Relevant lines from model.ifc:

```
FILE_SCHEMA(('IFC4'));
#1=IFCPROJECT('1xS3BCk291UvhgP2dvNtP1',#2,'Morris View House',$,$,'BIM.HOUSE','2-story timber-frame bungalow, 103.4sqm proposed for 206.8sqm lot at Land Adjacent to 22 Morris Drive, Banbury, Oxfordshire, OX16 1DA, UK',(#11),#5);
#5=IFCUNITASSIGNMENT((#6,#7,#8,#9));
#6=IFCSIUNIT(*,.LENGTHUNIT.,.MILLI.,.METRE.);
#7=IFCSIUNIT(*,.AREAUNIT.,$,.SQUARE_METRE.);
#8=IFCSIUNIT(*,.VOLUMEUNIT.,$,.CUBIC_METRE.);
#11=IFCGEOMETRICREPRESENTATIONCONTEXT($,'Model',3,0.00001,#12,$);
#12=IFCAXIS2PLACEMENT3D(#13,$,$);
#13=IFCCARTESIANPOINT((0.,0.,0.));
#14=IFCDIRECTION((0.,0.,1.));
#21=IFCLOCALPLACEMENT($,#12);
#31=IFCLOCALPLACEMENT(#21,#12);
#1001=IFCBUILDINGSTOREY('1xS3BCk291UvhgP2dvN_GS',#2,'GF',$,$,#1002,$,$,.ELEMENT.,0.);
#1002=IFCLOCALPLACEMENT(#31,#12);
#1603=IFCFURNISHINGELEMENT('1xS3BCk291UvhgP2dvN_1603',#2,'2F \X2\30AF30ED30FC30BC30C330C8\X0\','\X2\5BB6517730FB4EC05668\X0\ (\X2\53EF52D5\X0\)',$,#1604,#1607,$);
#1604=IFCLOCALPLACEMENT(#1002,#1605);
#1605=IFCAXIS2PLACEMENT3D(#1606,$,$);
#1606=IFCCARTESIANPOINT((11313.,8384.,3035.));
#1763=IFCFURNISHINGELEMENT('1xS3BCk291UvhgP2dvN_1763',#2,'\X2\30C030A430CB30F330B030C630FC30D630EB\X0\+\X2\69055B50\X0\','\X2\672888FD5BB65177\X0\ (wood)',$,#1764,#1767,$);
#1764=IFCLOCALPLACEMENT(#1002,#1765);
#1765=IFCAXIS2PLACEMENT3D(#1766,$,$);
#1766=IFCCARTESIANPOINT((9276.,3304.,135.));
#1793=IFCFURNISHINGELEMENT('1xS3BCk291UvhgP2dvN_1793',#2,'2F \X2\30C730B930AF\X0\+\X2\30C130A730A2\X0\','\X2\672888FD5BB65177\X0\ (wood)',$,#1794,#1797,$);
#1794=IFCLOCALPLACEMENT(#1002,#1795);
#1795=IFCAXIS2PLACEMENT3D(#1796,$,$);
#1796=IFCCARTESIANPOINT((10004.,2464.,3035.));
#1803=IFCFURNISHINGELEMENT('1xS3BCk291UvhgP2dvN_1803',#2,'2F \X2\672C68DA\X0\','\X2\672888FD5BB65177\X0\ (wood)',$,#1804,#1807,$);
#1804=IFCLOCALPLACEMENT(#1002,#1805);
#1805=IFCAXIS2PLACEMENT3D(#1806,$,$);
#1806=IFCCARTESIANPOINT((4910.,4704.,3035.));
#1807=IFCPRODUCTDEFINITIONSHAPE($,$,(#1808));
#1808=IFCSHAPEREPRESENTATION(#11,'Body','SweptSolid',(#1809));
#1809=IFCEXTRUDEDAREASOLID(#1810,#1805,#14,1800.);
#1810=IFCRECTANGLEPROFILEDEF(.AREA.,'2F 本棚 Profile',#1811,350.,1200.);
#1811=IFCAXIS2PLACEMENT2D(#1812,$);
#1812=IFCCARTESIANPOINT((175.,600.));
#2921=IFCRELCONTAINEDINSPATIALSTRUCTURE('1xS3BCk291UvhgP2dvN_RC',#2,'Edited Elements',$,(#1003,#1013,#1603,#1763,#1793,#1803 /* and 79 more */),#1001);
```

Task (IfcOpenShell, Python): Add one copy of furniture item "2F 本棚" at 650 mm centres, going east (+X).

```python
import numpy as np
import ifcopenshell
import ifcopenshell.api.geometry
import ifcopenshell.api.root
import ifcopenshell.util.element
import ifcopenshell.util.placement
import ifcopenshell.util.unit

model = ifcopenshell.open("model.ifc")
unit_scale = ifcopenshell.util.unit.calculate_unit_scale(model)


def reuse_history(source, copy):
    """copy_class also copies each property set's owner history, people and application; keep the originals."""
    for rel in copy.IsDefinedBy:
        if rel.is_a("IfcRelDefinesByProperties") and (history := rel.RelatingPropertyDefinition.OwnerHistory):
            rel.RelatingPropertyDefinition.OwnerHistory = source.OwnerHistory
            ifcopenshell.util.element.remove_deep2(model, history)


source = model.by_guid("1xS3BCk291UvhgP2dvN_1803")
base = ifcopenshell.util.placement.get_local_placement(source.ObjectPlacement)
step = np.array([1.0, 0.0, 0.0]) * 0.65 / unit_scale

for i in range(1, 2):
    copy = ifcopenshell.api.root.copy_class(model, product=source)
    copy.Representation = ifcopenshell.util.element.copy_deep(
        model, source.Representation, exclude=["IfcGeometricRepresentationContext", "IfcRepresentationMap"]
    )
    reuse_history(source, copy)
    matrix = base.copy()
    matrix[:3, 3] += i * step
    print("added at", matrix[:3, 3].round(3) + 0.0)
    ifcopenshell.api.geometry.edit_object_placement(model, product=copy, matrix=matrix, is_si=False)

model.write("model_updated.ifc")
```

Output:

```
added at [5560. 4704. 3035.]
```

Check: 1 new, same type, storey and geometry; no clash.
